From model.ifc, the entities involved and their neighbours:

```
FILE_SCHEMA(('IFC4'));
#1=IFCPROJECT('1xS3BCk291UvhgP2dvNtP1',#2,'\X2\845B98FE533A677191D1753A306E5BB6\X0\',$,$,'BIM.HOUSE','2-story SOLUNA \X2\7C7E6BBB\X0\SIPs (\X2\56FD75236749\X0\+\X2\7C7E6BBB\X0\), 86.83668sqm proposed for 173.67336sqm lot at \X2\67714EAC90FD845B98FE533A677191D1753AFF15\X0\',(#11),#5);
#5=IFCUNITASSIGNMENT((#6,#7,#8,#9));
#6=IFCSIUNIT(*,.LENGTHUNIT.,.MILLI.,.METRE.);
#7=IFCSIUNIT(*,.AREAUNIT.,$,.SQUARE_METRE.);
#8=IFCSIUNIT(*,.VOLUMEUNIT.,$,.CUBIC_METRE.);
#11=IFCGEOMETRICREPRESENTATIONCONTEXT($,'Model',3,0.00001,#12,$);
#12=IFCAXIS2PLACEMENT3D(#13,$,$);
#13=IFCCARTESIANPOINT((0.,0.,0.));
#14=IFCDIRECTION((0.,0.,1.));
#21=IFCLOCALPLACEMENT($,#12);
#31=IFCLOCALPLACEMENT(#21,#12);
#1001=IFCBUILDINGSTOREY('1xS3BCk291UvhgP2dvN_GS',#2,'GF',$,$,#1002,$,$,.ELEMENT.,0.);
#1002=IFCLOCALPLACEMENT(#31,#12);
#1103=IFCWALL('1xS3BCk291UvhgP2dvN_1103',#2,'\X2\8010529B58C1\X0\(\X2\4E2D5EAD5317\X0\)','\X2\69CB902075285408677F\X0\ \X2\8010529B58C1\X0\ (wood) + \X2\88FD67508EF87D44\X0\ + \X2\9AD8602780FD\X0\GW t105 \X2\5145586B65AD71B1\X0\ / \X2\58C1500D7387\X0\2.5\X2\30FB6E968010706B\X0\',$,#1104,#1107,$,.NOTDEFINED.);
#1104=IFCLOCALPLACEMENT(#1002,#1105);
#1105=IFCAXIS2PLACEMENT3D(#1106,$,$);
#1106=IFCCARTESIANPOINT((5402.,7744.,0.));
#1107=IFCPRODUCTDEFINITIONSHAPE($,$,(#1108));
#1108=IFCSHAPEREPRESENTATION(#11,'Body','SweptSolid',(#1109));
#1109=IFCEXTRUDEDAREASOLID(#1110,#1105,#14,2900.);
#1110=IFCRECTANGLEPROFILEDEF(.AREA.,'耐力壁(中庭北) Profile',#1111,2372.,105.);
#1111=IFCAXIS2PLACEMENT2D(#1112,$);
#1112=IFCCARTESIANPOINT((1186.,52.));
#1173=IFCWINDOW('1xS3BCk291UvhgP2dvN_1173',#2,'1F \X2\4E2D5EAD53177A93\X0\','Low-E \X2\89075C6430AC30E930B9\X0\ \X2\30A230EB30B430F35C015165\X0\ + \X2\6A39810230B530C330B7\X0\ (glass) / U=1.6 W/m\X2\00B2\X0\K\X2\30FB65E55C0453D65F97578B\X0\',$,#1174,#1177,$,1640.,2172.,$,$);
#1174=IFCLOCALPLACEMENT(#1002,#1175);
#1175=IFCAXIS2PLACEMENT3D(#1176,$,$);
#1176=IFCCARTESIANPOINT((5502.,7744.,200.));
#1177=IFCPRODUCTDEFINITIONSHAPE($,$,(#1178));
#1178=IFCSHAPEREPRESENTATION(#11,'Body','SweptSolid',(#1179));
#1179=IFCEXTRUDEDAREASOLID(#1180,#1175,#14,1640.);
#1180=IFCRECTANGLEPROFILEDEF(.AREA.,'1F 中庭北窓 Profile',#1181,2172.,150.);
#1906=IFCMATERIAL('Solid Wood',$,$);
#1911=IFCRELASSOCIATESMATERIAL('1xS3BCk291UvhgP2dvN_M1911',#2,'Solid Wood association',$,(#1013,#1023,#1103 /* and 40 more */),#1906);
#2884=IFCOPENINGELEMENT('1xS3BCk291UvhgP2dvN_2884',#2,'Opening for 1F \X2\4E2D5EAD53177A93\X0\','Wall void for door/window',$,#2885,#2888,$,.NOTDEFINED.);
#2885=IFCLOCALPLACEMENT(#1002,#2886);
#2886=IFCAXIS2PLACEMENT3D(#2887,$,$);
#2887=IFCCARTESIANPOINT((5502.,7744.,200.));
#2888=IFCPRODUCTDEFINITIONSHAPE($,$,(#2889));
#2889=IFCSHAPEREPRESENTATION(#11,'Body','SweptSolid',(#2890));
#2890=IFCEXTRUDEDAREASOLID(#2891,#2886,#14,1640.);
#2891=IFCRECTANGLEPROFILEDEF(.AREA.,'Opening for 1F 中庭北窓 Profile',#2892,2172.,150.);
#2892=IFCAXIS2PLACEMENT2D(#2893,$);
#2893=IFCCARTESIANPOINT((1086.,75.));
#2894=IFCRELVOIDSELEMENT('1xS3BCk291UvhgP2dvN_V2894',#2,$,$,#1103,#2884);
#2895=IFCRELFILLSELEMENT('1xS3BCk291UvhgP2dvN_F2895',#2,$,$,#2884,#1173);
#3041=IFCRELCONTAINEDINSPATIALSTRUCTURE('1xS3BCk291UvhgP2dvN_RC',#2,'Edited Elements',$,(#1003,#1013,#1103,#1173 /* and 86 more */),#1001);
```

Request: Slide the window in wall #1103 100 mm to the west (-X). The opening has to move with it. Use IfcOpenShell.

```python
import ifcopenshell
import ifcopenshell.api.geometry
import ifcopenshell.util.placement
import ifcopenshell.util.unit

model = ifcopenshell.open("model.ifc")
unit_scale = ifcopenshell.util.unit.calculate_unit_scale(model)

window = model.by_guid("1xS3BCk291UvhgP2dvN_1173")
opening = window.FillsVoids[0].RelatingOpeningElement
wall = opening.VoidsElements[0].RelatingBuildingElement

wall_matrix = ifcopenshell.util.placement.get_local_placement(wall.ObjectPlacement)
shift = wall_matrix[:3, 0] * -0.1 / unit_scale
before = ifcopenshell.util.placement.get_local_placement(window.ObjectPlacement)[:3, 3].copy()

# The window is not placed relative to its opening, so move both.
for product in (opening, window):
    matrix = ifcopenshell.util.placement.get_local_placement(product.ObjectPlacement)
    matrix[:3, 3] += shift
    ifcopenshell.api.geometry.edit_object_placement(model, product=product, matrix=matrix, is_si=False)

after = ifcopenshell.util.placement.get_local_placement(window.ObjectPlacement)[:3, 3]
print("window moved by", (after - before).round(3) + 0.0)

model.write("model_updated.ifc")
```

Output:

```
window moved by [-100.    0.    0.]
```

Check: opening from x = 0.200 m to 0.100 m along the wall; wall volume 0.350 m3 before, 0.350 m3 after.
